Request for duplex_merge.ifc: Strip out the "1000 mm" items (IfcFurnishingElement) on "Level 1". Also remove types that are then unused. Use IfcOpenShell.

First a look at what the model holds.

```python
import ifcopenshell
import ifcopenshell.util.element

model = ifcopenshell.open("duplex_merge.ifc")
print(model.schema)
storey = next(s for s in model.by_type("IfcBuildingStorey") if s.Name == "Level 1")
furniture = [e for e in ifcopenshell.util.element.get_decomposition(storey) if e.is_a("IfcFurnishingElement")]
seen = {}
for e in furniture:
    element_type = ifcopenshell.util.element.get_type(e)
    name = element_type.Name if element_type not in (None, e) else None
    seen[name] = seen.get(name, 0) + 1
for name, count in sorted(seen.items(), key=str):
    print(count, "x", name)
```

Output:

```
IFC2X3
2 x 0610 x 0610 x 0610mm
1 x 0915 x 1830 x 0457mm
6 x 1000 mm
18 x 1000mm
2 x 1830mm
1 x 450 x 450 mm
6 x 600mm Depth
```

```python
import ifcopenshell
import ifcopenshell.api.root
import ifcopenshell.util.element

model = ifcopenshell.open("duplex_merge.ifc")

storey = next(s for s in model.by_type("IfcBuildingStorey") if s.Name == "Level 1")
furniture = [e for e in ifcopenshell.util.element.get_decomposition(storey) if e.is_a("IfcFurnishingElement")]
targets = [e for e in furniture if (t := ifcopenshell.util.element.get_type(e)) not in (None, e) and t.Name == "1000 mm"]
types = {ifcopenshell.util.element.get_type(e) for e in targets} - {None, *targets}

for e in targets:
    ifcopenshell.api.root.remove_product(model, product=e)
print(len(targets), "removed")

unused = [t for t in types if not ifcopenshell.util.element.get_types(t)]
for t in unused:
    ifcopenshell.api.root.remove_product(model, product=t)
print(len(unused), "unused types removed")

model.write("duplex_merge_rev.ifc")
```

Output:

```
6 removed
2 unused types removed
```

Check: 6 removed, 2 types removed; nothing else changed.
